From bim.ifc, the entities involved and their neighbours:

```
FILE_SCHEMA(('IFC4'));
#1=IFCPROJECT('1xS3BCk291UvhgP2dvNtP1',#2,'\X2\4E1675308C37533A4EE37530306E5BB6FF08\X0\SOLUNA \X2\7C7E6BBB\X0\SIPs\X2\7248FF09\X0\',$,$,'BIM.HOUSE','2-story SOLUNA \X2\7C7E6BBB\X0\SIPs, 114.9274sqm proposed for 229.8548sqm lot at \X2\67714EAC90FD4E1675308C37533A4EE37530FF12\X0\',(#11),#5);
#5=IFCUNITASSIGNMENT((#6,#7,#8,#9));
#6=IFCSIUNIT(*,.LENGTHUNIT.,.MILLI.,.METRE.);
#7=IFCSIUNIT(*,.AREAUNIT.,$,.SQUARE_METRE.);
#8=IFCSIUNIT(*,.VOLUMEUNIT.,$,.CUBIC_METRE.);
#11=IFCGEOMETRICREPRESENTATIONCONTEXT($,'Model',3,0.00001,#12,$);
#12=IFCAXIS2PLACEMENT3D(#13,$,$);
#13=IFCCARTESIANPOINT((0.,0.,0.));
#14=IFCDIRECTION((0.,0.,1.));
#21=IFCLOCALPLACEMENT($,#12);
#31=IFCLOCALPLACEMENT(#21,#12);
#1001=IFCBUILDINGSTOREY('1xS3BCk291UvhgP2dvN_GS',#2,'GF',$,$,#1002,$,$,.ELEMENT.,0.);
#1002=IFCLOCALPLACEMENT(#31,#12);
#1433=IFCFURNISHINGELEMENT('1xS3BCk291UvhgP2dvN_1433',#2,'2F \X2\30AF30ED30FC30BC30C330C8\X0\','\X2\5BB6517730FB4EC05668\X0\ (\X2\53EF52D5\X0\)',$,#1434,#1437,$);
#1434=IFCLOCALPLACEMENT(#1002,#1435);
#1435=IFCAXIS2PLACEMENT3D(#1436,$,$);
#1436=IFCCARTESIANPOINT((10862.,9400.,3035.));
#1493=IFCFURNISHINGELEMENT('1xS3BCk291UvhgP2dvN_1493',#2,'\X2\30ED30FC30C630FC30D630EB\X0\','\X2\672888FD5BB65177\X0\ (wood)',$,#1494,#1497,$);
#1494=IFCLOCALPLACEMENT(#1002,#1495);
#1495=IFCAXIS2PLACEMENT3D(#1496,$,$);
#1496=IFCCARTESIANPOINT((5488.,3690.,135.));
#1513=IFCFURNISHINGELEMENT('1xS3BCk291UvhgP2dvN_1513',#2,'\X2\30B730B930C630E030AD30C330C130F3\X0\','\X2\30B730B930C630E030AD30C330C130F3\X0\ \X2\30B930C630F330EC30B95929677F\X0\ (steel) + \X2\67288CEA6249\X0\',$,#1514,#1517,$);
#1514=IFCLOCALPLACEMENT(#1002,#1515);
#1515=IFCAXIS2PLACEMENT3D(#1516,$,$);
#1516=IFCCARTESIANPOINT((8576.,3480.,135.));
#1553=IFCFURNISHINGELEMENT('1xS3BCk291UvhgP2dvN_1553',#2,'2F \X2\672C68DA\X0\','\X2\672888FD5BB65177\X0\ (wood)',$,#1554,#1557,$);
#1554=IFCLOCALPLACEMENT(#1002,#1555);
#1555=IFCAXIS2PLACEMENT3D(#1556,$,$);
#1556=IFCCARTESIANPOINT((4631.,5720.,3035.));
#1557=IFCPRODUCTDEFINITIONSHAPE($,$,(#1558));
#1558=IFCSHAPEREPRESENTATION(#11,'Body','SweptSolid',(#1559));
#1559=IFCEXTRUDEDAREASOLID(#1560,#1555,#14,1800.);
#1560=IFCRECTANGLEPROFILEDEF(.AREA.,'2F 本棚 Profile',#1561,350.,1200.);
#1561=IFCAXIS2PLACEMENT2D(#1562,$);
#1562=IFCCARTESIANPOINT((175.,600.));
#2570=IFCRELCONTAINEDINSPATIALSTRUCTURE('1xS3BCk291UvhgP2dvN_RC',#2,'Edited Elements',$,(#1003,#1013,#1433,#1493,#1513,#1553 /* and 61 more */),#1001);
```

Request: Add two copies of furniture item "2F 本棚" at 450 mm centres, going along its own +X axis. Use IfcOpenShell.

```python
import ifcopenshell
import ifcopenshell.api.geometry
import ifcopenshell.api.root
import ifcopenshell.util.element
import ifcopenshell.util.placement

model = ifcopenshell.open("bim.ifc")


def reuse_history(source, copy):
    """copy_class also copies each property set's owner history, people and application; keep the originals."""
    for rel in copy.IsDefinedBy:
        if rel.is_a("IfcRelDefinesByProperties") and (history := rel.RelatingPropertyDefinition.OwnerHistory):
            rel.RelatingPropertyDefinition.OwnerHistory = source.OwnerHistory
            ifcopenshell.util.element.remove_deep2(model, history)


source = model.by_guid("1xS3BCk291UvhgP2dvN_1553")
base = ifcopenshell.util.placement.get_local_placement(source.ObjectPlacement)
step = base[:3, 0] * 450.0

for i in range(1, 3):
    copy = ifcopenshell.api.root.copy_class(model, product=source)
    copy.Representation = ifcopenshell.util.element.copy_deep(
        model, source.Representation, exclude=["IfcGeometricRepresentationContext", "IfcRepresentationMap"]
    )
    reuse_history(source, copy)
    matrix = base.copy()
    matrix[:3, 3] += i * step
    print("added at", matrix[:3, 3].round(3) + 0.0)
    ifcopenshell.api.geometry.edit_object_placement(model, product=copy, matrix=matrix, is_si=False)

model.write("bim_updated.ifc")
```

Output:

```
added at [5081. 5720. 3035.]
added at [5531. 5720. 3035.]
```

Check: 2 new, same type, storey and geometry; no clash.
